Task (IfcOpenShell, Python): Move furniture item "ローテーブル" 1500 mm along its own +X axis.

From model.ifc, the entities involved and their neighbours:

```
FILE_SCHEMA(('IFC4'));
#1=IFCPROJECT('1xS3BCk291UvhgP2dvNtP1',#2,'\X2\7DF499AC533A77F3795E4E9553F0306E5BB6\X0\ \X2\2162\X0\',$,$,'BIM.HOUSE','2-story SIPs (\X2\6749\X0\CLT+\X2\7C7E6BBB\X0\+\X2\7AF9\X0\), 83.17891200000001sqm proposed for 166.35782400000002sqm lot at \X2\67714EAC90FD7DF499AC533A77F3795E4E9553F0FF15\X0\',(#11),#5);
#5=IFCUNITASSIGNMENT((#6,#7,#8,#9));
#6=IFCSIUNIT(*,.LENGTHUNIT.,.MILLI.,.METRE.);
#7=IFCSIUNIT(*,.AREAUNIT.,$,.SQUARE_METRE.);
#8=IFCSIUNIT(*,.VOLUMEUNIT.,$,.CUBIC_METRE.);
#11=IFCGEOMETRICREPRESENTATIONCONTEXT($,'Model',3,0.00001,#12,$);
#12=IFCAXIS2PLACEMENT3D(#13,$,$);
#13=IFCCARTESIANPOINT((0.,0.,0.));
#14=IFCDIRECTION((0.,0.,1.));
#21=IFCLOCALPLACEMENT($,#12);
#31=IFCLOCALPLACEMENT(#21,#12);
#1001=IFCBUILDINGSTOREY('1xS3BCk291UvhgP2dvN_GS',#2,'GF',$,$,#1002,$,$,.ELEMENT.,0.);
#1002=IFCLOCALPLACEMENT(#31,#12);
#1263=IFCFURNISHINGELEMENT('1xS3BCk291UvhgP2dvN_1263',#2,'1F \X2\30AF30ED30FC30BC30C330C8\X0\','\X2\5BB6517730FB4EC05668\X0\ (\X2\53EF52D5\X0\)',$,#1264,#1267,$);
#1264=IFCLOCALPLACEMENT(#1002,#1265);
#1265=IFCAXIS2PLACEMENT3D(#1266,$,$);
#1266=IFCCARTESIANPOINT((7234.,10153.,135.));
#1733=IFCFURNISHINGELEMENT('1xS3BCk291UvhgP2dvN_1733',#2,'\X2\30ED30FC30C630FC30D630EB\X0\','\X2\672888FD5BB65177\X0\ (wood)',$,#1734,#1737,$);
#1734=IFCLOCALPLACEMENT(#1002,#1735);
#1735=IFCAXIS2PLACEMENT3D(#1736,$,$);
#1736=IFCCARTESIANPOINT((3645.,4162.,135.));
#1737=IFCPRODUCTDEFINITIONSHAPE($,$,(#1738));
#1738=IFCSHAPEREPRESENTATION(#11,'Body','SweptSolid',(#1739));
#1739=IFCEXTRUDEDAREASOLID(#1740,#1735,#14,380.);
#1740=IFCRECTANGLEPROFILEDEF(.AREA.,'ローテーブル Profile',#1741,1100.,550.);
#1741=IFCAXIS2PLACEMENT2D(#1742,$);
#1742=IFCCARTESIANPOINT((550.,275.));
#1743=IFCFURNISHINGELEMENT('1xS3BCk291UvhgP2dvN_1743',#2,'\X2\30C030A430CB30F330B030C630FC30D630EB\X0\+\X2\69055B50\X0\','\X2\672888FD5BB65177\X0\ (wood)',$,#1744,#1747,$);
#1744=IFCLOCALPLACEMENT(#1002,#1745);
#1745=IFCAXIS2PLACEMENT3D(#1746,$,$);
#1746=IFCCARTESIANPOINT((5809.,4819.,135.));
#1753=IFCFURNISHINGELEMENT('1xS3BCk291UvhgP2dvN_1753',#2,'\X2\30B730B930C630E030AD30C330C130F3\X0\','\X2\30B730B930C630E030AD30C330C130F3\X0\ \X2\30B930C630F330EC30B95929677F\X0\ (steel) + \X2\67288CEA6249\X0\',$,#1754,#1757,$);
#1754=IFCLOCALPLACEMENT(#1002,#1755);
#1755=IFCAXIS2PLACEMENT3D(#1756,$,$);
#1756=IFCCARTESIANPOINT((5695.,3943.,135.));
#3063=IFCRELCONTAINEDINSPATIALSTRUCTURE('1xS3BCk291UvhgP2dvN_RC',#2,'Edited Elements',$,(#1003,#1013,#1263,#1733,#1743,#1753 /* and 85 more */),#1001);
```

```python
import ifcopenshell
import ifcopenshell.api.geometry
import ifcopenshell.util.placement
import ifcopenshell.util.unit

model = ifcopenshell.open("model.ifc")
unit_scale = ifcopenshell.util.unit.calculate_unit_scale(model)

item = model.by_guid("1xS3BCk291UvhgP2dvN_1733")
matrix = ifcopenshell.util.placement.get_local_placement(item.ObjectPlacement)
matrix[:3, 3] += matrix[:3, 0] * 1.5 / unit_scale
ifcopenshell.api.geometry.edit_object_placement(model, product=item, matrix=matrix, is_si=False)

print(ifcopenshell.util.placement.get_local_placement(item.ObjectPlacement).round(3) + 0.0)

model.write("model_rev.ifc")
```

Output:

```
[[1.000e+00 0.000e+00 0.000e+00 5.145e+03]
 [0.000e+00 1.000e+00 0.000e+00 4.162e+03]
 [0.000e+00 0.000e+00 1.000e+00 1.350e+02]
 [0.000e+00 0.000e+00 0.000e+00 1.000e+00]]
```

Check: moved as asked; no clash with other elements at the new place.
